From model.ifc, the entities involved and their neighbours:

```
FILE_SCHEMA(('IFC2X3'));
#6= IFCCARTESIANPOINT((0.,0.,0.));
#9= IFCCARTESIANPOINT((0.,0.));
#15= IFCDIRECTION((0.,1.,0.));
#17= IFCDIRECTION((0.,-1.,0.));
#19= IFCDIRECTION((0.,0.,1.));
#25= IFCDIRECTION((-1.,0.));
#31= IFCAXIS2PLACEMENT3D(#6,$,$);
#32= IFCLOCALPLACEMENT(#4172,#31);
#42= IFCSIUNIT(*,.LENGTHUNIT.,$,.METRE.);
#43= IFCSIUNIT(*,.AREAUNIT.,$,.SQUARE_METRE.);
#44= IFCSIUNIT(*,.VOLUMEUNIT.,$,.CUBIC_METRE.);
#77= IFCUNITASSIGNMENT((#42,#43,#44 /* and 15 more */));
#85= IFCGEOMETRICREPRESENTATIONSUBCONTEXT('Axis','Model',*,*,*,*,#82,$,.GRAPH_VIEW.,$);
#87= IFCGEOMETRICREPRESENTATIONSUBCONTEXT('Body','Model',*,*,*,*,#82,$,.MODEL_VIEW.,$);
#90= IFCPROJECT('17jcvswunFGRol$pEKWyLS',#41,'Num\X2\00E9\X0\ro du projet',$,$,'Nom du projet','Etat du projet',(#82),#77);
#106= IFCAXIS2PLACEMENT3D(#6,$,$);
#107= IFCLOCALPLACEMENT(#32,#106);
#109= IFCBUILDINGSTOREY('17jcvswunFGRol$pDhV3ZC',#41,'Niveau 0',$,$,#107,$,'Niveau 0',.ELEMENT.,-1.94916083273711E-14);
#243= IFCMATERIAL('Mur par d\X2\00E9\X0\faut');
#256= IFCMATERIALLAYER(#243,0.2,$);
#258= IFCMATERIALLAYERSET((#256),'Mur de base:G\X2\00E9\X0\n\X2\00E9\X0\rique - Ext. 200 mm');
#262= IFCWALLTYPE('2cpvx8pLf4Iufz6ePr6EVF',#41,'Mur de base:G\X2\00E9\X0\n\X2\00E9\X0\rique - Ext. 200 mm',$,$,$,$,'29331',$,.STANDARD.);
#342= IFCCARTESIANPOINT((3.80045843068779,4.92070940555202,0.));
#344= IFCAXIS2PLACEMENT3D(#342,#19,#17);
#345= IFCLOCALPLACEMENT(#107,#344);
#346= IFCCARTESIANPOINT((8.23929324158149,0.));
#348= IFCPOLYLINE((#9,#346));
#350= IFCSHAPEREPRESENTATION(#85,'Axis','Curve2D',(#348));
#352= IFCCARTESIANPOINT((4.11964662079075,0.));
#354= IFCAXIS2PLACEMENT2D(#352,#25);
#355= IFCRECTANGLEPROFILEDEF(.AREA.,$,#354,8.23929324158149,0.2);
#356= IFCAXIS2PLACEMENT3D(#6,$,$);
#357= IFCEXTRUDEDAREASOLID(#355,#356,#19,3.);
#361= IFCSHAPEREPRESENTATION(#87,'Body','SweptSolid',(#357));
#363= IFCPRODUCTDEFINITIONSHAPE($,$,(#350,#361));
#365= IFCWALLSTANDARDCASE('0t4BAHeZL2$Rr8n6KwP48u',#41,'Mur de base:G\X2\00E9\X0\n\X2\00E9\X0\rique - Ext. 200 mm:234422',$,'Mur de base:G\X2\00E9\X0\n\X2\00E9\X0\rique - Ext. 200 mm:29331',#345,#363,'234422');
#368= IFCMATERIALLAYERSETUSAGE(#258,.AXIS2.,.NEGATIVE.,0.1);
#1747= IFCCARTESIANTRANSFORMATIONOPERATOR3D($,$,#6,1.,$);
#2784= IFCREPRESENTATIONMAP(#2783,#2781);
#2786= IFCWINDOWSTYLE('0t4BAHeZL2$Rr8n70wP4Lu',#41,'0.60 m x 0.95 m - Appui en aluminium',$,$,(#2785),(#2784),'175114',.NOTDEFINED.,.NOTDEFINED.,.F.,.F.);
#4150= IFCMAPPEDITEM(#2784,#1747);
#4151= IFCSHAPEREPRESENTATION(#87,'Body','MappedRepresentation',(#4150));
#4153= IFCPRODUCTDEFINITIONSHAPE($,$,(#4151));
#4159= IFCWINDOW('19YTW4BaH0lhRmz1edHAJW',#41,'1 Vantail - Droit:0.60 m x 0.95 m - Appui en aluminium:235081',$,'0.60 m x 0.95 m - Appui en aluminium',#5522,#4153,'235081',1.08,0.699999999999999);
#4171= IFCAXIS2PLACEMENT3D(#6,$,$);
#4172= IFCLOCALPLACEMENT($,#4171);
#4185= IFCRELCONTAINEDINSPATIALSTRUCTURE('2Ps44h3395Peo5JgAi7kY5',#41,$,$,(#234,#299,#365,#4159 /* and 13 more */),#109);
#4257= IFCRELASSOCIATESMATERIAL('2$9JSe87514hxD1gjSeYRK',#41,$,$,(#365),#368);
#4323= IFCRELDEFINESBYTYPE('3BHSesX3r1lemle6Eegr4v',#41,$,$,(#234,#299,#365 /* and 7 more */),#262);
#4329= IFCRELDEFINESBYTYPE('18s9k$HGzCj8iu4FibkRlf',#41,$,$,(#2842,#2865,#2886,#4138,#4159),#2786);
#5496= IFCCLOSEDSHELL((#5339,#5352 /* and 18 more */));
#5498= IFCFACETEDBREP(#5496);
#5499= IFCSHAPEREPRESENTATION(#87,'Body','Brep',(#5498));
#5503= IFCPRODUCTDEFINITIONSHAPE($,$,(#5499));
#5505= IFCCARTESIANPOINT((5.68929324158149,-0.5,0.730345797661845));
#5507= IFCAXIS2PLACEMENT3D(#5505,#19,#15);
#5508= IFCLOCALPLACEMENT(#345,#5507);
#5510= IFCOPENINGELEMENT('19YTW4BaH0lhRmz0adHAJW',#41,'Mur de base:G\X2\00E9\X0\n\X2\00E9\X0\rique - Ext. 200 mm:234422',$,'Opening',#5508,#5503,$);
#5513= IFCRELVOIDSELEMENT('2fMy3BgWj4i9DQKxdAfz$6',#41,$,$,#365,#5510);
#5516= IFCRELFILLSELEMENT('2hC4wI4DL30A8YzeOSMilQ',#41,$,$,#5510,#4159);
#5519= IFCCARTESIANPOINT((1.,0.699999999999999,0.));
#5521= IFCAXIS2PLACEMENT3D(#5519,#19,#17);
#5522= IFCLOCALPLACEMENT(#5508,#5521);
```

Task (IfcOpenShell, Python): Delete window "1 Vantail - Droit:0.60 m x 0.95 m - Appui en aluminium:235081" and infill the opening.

```python
import ifcopenshell
import ifcopenshell.api.feature
import ifcopenshell.api.root
import ifcopenshell.geom
import ifcopenshell.util.shape

model = ifcopenshell.open("model.ifc")
settings = ifcopenshell.geom.settings()


def volume(element):
    """Net volume in cubic metres, openings subtracted."""
    shape = ifcopenshell.geom.create_shape(settings, element)
    return ifcopenshell.util.shape.get_volume(shape.geometry)


window = model.by_id(4159)
opening = window.FillsVoids[0].RelatingOpeningElement
wall = opening.VoidsElements[0].RelatingBuildingElement
before = volume(wall)

ifcopenshell.api.root.remove_product(model, product=window)
ifcopenshell.api.feature.remove_feature(model, feature=opening)

after = volume(wall)

print(f"wall volume {before:.3f} -> {after:.3f} m3")

model.write("model-out.ifc")
```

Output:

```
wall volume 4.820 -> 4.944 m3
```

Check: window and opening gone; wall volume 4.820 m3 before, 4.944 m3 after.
